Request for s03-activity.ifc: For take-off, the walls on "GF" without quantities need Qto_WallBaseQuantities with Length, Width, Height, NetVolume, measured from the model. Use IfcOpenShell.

First a look at what the model holds.

```python
import ifcopenshell
import ifcopenshell.util.element
import ifcopenshell.util.unit

model = ifcopenshell.open("s03-activity.ifc")
print(model.schema)
for unit_type in ("LENGTHUNIT", "AREAUNIT", "VOLUMEUNIT"):
    print(unit_type, ifcopenshell.util.unit.calculate_unit_scale(model, unit_type))
storey = next(s for s in model.by_type("IfcBuildingStorey") if s.Name == "GF")
walls = [e for e in ifcopenshell.util.element.get_decomposition(storey) if e.is_a("IfcWall")]
for e in sorted(walls, key=lambda e: e.id()):
    print(e.id(), e.is_a(), e.Name, list(ifcopenshell.util.element.get_psets(e, qtos_only=True)), sep=" | ")
```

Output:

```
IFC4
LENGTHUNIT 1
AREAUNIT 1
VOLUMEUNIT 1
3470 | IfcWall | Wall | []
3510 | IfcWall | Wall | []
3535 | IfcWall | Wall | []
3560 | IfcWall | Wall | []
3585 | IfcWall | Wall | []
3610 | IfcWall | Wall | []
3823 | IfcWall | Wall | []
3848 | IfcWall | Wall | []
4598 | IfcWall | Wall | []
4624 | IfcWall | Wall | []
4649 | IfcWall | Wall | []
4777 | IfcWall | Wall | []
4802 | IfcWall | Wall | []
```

```python
import ifcopenshell
import ifcopenshell.api.pset
import ifcopenshell.geom
import ifcopenshell.util.element
import ifcopenshell.util.shape
import ifcopenshell.util.unit

model = ifcopenshell.open("s03-activity.ifc")
unit_scale = ifcopenshell.util.unit.calculate_unit_scale(model)
volume_scale = ifcopenshell.util.unit.calculate_unit_scale(model, "VOLUMEUNIT")
settings = ifcopenshell.geom.settings()

storey = next(s for s in model.by_type("IfcBuildingStorey") if s.Name == "GF")
walls = [e for e in ifcopenshell.util.element.get_decomposition(storey) if e.is_a("IfcWall")]

for e in sorted(walls, key=lambda e: e.id()):
    if ifcopenshell.util.element.get_psets(e, qtos_only=True, should_inherit=False):
        continue
    # Geometry comes back in metres, in the element's own axes.
    shape = ifcopenshell.geom.create_shape(settings, e)
    values = {
        "Length": ifcopenshell.util.shape.get_x(shape.geometry) / unit_scale,
        "Width": ifcopenshell.util.shape.get_y(shape.geometry) / unit_scale,
        "Height": ifcopenshell.util.shape.get_z(shape.geometry) / unit_scale,
        "NetVolume": ifcopenshell.util.shape.get_volume(shape.geometry) / volume_scale,
    }
    qto = ifcopenshell.api.pset.add_qto(model, product=e, name="Qto_WallBaseQuantities")
    ifcopenshell.api.pset.edit_qto(model, qto=qto, properties=values)
    print(e.id(), {k: round(v, 3) for k, v in values.items()})

model.write("s03-activity_edited.ifc")
```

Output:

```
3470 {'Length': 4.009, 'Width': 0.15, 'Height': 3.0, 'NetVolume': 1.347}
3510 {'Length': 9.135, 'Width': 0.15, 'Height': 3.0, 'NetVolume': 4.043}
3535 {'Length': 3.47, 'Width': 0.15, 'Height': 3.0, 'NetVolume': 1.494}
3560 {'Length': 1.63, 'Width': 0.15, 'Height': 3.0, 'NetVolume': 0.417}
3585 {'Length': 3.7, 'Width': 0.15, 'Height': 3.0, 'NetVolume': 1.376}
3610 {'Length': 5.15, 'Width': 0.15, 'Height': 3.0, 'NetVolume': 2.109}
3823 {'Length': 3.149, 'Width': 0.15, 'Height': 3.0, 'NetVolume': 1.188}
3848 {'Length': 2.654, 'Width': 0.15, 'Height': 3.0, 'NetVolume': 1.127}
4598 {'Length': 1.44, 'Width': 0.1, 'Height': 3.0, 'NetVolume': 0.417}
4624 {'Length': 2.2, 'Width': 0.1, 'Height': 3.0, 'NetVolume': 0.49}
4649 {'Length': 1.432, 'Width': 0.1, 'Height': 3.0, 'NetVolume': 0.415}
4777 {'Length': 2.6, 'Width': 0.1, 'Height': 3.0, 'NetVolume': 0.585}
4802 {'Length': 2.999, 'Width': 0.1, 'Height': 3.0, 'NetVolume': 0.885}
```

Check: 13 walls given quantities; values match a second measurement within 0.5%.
